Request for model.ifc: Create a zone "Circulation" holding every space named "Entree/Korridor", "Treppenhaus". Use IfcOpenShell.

First a look at what the model holds.

```python
import ifcopenshell

model = ifcopenshell.open("model.ifc")
print(model.schema)
seen = {}
for space in model.by_type("IfcSpace"):
    seen[space.LongName] = seen.get(space.LongName, 0) + 1
for name, count in sorted(seen.items(), key=str):
    print(count, "x", name)
print("zones:", [z.Name for z in model.by_type("IfcZone")][:20])
```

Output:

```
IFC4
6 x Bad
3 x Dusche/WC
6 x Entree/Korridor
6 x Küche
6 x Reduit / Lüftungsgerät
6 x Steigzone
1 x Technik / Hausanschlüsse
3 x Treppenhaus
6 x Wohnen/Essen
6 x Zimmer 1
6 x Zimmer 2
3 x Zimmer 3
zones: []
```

```python
import ifcopenshell
import ifcopenshell.api.group
import ifcopenshell.api.root

model = ifcopenshell.open("model.ifc")

names = {"Entree/Korridor", "Treppenhaus"}
spaces = [s for s in model.by_type("IfcSpace") if s.LongName in names]

zone = ifcopenshell.api.root.create_entity(model, ifc_class="IfcZone", name="Circulation")
ifcopenshell.api.group.assign_group(model, products=spaces, group=zone)
print(len(spaces), "spaces in", zone.Name)

model.write("model_edited.ifc")
```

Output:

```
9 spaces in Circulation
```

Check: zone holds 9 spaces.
